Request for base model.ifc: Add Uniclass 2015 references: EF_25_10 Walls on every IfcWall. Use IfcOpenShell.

First a look at what the model holds.

```python
import ifcopenshell

model = ifcopenshell.open("base model.ifc")
print(model.schema)
print("classifications:", [c.Name for c in model.by_type("IfcClassification")])
for ifc_class in ("IfcDoor", "IfcRoof", "IfcStair", "IfcWall", "IfcWindow"):
    print(ifc_class, len(model.by_type(ifc_class)))
```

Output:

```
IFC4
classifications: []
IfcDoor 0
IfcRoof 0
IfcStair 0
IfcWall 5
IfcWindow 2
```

```python
import ifcopenshell
import ifcopenshell.api.classification

model = ifcopenshell.open("base model.ifc")

system = ifcopenshell.api.classification.add_classification(model, classification="Uniclass 2015")

codes = {
    "IfcWall": ("EF_25_10", "Walls"),
}
for ifc_class, (code, name) in codes.items():
    products = model.by_type(ifc_class)
    ifcopenshell.api.classification.add_reference(
        model, products=products, classification=system, identification=code, name=name
    )
    print(code, len(products))

model.write("base model_updated.ifc")
```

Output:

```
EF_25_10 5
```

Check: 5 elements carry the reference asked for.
